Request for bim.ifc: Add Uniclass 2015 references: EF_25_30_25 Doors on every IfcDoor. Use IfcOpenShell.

First a look at what the model holds.

```python
import ifcopenshell

model = ifcopenshell.open("bim.ifc")
print(model.schema)
print("classifications:", [c.Name for c in model.by_type("IfcClassification")])
for ifc_class in ("IfcDoor", "IfcRoof", "IfcStair", "IfcWall", "IfcWindow"):
    print(ifc_class, len(model.by_type(ifc_class)))
```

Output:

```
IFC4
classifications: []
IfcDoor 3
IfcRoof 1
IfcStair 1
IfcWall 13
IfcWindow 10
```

```python
import ifcopenshell
import ifcopenshell.api.classification

model = ifcopenshell.open("bim.ifc")

system = ifcopenshell.api.classification.add_classification(model, classification="Uniclass 2015")

codes = {
    "IfcDoor": ("EF_25_30_25", "Doors"),
}
for ifc_class, (code, name) in codes.items():
    products = model.by_type(ifc_class)
    ifcopenshell.api.classification.add_reference(
        model, products=products, classification=system, identification=code, name=name
    )
    print(code, len(products))

model.write("bim_edited.ifc")
```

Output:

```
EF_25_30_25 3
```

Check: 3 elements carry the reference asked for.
